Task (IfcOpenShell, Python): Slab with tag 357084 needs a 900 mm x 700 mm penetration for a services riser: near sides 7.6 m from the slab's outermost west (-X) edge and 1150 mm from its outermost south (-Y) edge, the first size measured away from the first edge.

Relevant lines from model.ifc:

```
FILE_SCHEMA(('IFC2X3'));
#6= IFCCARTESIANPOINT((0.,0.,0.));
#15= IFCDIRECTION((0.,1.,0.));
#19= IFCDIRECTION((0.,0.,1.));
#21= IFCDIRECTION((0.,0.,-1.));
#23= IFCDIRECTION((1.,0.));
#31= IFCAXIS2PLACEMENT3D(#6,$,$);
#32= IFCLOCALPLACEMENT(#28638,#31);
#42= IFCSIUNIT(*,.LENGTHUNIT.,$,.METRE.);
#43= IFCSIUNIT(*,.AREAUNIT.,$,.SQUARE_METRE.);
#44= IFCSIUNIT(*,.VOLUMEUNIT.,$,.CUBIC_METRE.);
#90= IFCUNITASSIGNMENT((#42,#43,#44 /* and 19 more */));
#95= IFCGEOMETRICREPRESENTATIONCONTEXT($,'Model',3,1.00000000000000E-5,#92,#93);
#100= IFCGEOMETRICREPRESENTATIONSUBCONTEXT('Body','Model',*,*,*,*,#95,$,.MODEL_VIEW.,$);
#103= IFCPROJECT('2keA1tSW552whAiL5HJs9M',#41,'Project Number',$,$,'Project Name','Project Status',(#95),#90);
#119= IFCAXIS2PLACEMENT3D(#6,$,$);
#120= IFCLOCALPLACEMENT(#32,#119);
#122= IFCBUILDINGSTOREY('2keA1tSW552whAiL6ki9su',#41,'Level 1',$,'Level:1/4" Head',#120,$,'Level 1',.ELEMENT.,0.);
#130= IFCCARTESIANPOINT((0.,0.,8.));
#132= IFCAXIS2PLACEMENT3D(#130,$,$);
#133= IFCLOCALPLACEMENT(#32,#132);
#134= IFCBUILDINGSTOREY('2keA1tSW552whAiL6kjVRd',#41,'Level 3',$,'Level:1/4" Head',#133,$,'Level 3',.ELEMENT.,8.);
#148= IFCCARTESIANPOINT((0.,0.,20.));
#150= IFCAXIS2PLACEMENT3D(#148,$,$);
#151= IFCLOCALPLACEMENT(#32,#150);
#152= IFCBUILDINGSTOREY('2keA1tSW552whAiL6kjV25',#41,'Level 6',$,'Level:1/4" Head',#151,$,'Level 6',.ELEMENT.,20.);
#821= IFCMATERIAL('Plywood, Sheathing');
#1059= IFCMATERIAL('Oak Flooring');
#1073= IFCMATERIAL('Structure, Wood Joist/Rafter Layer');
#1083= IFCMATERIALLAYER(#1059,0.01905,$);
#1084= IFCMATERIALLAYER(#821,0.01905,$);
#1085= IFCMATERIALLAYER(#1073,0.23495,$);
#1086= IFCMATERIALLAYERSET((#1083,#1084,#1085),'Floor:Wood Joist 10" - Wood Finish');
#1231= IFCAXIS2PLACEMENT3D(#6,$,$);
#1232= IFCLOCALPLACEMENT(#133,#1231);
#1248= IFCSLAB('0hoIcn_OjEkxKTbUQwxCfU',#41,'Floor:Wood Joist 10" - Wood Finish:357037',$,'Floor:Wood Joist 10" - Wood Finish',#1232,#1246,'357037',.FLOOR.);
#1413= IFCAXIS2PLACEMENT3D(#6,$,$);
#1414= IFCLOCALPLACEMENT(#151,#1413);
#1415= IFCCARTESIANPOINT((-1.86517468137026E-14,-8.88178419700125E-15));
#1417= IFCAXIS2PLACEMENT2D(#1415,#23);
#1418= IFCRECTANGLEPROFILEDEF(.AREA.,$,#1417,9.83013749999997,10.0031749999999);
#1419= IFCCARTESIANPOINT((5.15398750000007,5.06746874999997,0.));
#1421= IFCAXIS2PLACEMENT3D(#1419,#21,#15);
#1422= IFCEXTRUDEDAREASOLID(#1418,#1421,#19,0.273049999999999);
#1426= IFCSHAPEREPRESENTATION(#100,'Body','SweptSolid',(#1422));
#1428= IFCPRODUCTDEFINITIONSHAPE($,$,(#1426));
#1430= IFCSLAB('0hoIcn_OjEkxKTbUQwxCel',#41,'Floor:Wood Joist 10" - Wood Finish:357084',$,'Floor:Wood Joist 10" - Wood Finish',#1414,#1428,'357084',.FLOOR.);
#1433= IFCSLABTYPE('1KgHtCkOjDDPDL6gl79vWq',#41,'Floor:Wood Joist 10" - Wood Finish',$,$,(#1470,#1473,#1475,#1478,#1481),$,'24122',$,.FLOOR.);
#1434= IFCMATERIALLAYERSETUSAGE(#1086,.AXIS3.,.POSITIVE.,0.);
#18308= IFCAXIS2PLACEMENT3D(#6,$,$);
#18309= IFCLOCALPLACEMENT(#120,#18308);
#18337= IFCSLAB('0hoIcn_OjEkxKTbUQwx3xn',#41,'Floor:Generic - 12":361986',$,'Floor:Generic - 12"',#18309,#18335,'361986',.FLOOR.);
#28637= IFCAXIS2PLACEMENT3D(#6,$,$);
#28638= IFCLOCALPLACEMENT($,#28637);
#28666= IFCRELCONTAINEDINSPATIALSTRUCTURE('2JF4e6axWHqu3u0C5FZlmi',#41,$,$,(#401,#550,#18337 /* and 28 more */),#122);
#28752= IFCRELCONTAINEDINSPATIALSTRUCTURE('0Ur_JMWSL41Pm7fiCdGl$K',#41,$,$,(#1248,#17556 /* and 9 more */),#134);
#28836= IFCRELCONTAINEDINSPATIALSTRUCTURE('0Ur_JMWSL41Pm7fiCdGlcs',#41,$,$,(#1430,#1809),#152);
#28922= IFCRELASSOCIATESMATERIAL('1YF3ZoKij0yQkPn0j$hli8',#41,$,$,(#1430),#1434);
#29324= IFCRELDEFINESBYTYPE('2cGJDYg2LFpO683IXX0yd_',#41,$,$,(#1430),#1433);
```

```python
import numpy as np
import ifcopenshell
import ifcopenshell.api.feature
import ifcopenshell.api.geometry
import ifcopenshell.api.root
import ifcopenshell.geom
import ifcopenshell.util.placement
import ifcopenshell.util.representation
import ifcopenshell.util.shape
import ifcopenshell.util.unit

model = ifcopenshell.open("model.ifc")
unit_scale = ifcopenshell.util.unit.calculate_unit_scale(model)
settings = ifcopenshell.geom.settings()


def volume(element):
    """Net volume in cubic metres, openings subtracted."""
    shape = ifcopenshell.geom.create_shape(settings, element)
    return ifcopenshell.util.shape.get_volume(shape.geometry)


slab = model.by_guid("0hoIcn_OjEkxKTbUQwxCel")
before = volume(slab)

# Extent in the slab's own axes, in metres. The edges named are its -X and -Y sides.
slab_shape = ifcopenshell.geom.create_shape(settings, slab)
vertices = ifcopenshell.util.shape.get_vertices(slab_shape.geometry)
x_min, y_min, bottom = vertices.min(axis=0)
top = vertices[:, 2].max()

opening = ifcopenshell.api.root.create_entity(model, ifc_class="IfcOpeningElement", name="Services riser opening")
context = ifcopenshell.util.representation.get_context(model, "Model", "Body", "MODEL_VIEW")
width, depth = 0.9, 0.7
outline = [(0.0, 0.0), (width, 0.0), (width, depth), (0.0, depth), (0.0, 0.0)]
# Overshoot both faces by 50 mm so the cut is clean.
shape = ifcopenshell.api.geometry.add_slab_representation(
    model, context=context, depth=top - bottom + 0.1, polyline=outline
)
ifcopenshell.api.geometry.assign_representation(model, product=opening, representation=shape)

matrix = ifcopenshell.util.placement.get_local_placement(slab.ObjectPlacement)
matrix[:, 3] = matrix @ np.append(np.array([x_min + 7.6, y_min + 1.15, bottom - 0.05]) / unit_scale, 1.0)
ifcopenshell.api.geometry.edit_object_placement(model, product=opening, matrix=matrix, is_si=False)
ifcopenshell.api.feature.add_feature(model, feature=opening, element=slab)

after = volume(slab)

print(f"slab volume {before:.3f} -> {after:.3f} m3")

model.write("model-out.ifc")
```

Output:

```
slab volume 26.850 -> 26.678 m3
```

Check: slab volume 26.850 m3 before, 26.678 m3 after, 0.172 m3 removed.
